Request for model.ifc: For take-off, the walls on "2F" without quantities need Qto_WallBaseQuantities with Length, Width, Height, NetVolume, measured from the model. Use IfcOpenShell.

First a look at what the model holds.

```python
import ifcopenshell
import ifcopenshell.util.element
import ifcopenshell.util.unit

model = ifcopenshell.open("model.ifc")
print(model.schema)
for unit_type in ("LENGTHUNIT", "AREAUNIT", "VOLUMEUNIT"):
    print(unit_type, ifcopenshell.util.unit.calculate_unit_scale(model, unit_type))
storey = next(s for s in model.by_type("IfcBuildingStorey") if s.Name == "2F")
walls = [e for e in ifcopenshell.util.element.get_decomposition(storey) if e.is_a("IfcWall")]
for e in sorted(walls, key=lambda e: e.id()):
    print(e.id(), e.is_a(), e.Name, list(ifcopenshell.util.element.get_psets(e, qtos_only=True)), sep=" | ")
```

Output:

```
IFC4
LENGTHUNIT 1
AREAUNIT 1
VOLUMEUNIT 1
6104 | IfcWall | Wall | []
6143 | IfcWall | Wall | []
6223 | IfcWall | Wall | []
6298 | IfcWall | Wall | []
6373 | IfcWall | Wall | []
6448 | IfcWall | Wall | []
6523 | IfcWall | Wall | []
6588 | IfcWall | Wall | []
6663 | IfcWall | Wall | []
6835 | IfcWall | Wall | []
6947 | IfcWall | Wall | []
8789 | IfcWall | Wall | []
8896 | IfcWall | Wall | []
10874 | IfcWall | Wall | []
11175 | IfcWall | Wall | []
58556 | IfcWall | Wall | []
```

```python
import ifcopenshell
import ifcopenshell.api.pset
import ifcopenshell.geom
import ifcopenshell.util.element
import ifcopenshell.util.shape
import ifcopenshell.util.unit

model = ifcopenshell.open("model.ifc")
unit_scale = ifcopenshell.util.unit.calculate_unit_scale(model)
volume_scale = ifcopenshell.util.unit.calculate_unit_scale(model, "VOLUMEUNIT")
settings = ifcopenshell.geom.settings()

storey = next(s for s in model.by_type("IfcBuildingStorey") if s.Name == "2F")
walls = [e for e in ifcopenshell.util.element.get_decomposition(storey) if e.is_a("IfcWall")]

for e in sorted(walls, key=lambda e: e.id()):
    if ifcopenshell.util.element.get_psets(e, qtos_only=True, should_inherit=False):
        continue
    # Geometry comes back in metres, in the element's own axes.
    shape = ifcopenshell.geom.create_shape(settings, e)
    values = {
        "Length": ifcopenshell.util.shape.get_x(shape.geometry) / unit_scale,
        "Width": ifcopenshell.util.shape.get_y(shape.geometry) / unit_scale,
        "Height": ifcopenshell.util.shape.get_z(shape.geometry) / unit_scale,
        "NetVolume": ifcopenshell.util.shape.get_volume(shape.geometry) / volume_scale,
    }
    qto = ifcopenshell.api.pset.add_qto(model, product=e, name="Qto_WallBaseQuantities")
    ifcopenshell.api.pset.edit_qto(model, qto=qto, properties=values)
    print(e.id(), {k: round(v, 3) for k, v in values.items()})

model.write("model_updated.ifc")
```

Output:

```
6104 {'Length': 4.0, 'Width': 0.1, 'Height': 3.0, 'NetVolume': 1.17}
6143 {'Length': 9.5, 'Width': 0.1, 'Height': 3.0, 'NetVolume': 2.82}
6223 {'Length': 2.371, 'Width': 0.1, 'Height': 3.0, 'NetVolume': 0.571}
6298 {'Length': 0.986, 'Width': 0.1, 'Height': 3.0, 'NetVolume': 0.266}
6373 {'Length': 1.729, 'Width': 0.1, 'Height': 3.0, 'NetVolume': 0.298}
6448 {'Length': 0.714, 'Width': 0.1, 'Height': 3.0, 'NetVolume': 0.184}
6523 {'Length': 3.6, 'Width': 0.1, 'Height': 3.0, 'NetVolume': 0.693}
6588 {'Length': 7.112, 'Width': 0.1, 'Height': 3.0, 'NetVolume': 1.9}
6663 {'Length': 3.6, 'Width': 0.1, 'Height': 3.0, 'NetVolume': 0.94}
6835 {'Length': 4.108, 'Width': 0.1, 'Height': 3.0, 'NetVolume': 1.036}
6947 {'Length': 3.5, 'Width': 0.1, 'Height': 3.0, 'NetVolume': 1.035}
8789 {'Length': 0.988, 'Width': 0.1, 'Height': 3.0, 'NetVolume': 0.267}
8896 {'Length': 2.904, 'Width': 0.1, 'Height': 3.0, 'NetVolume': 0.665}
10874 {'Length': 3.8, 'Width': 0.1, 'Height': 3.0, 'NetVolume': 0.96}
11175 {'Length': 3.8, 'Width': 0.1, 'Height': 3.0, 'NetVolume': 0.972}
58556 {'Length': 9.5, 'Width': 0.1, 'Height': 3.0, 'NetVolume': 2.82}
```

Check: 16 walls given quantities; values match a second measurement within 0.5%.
